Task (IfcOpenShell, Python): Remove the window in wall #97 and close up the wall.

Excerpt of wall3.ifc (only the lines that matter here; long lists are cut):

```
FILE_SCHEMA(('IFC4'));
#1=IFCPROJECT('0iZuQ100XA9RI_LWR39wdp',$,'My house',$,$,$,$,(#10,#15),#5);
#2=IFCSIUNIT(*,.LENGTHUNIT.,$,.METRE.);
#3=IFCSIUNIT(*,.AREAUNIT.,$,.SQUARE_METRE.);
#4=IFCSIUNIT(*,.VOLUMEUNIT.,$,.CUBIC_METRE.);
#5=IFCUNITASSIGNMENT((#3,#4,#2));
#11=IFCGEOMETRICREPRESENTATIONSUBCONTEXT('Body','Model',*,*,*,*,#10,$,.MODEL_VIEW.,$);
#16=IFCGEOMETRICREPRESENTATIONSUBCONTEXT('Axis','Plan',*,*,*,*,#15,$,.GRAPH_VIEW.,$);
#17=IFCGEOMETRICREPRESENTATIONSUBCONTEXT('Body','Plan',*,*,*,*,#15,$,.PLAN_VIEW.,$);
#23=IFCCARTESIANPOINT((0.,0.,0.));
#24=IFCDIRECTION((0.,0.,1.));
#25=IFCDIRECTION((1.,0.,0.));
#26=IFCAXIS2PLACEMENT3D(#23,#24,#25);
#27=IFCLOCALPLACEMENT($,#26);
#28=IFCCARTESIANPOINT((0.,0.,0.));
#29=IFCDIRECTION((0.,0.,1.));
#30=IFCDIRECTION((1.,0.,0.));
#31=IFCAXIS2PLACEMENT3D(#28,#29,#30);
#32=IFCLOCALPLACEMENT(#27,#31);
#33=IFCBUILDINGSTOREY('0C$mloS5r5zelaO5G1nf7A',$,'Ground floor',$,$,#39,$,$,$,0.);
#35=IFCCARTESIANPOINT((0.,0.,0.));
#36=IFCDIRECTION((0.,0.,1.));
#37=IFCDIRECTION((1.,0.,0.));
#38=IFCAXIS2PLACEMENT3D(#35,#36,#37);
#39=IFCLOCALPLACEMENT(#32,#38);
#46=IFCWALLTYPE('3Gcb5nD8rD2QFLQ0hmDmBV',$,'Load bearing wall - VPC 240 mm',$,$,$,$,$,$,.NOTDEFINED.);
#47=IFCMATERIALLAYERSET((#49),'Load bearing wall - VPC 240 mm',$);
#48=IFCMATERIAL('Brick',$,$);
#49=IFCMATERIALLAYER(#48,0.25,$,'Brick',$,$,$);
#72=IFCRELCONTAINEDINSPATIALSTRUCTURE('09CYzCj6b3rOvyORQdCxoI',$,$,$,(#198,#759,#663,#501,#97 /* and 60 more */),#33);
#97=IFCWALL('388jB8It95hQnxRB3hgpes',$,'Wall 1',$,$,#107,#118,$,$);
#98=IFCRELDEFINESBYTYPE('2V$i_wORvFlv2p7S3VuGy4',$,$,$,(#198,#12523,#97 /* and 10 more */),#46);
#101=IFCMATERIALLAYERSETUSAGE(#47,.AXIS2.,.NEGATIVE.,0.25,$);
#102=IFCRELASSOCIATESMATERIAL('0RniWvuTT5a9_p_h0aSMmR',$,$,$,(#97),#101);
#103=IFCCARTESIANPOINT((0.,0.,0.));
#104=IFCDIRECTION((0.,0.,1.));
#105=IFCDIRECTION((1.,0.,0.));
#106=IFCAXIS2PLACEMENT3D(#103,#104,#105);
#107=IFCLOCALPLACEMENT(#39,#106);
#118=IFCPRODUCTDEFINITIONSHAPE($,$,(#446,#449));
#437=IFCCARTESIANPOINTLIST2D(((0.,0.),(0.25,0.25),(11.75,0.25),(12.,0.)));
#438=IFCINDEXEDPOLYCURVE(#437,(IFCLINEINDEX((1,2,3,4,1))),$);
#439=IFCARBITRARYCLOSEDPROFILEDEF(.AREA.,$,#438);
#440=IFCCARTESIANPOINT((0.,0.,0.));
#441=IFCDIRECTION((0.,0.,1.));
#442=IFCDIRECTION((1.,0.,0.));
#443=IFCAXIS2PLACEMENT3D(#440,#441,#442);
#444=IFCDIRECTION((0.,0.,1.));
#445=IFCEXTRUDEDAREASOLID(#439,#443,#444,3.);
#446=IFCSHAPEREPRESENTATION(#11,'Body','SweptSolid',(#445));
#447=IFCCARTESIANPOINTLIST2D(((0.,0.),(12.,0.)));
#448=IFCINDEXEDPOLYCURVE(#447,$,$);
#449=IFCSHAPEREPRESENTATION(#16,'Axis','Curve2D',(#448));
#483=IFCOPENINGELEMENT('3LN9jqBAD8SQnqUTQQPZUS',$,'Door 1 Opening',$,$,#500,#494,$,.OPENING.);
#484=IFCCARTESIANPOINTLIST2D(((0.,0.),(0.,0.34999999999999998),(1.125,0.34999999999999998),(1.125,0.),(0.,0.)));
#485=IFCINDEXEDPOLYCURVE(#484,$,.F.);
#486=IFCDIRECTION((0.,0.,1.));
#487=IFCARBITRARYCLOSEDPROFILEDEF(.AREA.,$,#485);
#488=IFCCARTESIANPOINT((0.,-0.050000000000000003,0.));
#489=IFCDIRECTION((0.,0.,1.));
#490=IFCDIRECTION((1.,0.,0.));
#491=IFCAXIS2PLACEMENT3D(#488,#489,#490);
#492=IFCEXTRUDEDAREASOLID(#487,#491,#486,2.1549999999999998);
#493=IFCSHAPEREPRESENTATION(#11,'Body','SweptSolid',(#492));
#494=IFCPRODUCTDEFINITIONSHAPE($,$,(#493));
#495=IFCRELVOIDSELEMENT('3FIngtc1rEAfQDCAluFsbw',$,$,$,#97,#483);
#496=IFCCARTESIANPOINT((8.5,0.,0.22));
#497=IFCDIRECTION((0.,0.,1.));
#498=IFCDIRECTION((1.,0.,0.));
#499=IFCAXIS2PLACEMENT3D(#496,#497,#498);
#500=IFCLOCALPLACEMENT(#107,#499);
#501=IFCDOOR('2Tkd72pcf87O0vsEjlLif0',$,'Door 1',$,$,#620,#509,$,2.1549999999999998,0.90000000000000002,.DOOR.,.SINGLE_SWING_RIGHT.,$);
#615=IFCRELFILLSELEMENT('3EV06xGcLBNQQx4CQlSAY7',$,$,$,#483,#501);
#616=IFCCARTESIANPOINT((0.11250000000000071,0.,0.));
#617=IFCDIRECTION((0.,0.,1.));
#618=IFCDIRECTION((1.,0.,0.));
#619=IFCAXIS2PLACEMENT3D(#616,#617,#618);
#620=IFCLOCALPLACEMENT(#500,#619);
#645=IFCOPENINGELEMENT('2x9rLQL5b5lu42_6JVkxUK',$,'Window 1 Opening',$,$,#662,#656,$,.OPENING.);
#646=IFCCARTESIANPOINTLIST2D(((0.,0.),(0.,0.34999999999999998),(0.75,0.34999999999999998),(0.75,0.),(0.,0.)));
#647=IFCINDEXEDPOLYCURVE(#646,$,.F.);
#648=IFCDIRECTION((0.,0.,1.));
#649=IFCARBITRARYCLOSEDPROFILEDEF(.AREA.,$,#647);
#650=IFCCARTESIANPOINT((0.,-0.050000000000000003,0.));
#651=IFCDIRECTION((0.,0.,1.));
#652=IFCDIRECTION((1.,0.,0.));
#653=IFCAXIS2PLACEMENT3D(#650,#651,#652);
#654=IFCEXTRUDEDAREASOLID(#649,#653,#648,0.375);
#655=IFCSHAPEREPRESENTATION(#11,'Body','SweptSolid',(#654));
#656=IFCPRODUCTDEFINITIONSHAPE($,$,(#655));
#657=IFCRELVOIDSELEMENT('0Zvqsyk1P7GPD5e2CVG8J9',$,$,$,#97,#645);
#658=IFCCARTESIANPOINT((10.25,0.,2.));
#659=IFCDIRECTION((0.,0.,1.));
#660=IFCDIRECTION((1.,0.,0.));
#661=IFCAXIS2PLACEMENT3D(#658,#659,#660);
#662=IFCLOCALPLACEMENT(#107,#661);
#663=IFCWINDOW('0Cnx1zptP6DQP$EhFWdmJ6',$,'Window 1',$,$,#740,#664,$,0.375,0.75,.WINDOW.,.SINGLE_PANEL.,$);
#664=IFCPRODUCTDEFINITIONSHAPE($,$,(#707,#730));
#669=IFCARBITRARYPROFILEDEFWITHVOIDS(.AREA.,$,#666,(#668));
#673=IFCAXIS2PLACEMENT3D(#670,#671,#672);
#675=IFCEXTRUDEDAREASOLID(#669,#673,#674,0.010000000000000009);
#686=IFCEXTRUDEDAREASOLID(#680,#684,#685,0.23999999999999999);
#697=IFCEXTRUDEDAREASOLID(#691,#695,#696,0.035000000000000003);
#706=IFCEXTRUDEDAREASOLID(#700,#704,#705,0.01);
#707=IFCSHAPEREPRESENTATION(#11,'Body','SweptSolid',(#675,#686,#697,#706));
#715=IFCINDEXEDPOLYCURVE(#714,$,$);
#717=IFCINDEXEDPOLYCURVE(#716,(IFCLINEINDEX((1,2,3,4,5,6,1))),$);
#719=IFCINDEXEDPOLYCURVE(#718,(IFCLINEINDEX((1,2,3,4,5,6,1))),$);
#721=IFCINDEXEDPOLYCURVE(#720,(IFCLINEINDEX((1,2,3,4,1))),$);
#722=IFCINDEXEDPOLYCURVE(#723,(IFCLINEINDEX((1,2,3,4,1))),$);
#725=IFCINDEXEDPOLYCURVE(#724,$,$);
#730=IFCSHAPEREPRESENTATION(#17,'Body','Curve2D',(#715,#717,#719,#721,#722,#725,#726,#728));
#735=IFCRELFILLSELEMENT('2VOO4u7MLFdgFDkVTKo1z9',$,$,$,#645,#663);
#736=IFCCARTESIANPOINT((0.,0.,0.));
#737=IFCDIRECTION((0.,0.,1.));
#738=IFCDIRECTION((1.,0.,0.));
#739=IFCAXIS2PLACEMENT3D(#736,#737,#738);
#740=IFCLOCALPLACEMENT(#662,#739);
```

```python
import ifcopenshell
import ifcopenshell.api.feature
import ifcopenshell.api.root
import ifcopenshell.geom
import ifcopenshell.util.shape

model = ifcopenshell.open("wall3.ifc")
settings = ifcopenshell.geom.settings()


def volume(element):
    """Net volume in cubic metres, openings subtracted."""
    shape = ifcopenshell.geom.create_shape(settings, element)
    return ifcopenshell.util.shape.get_volume(shape.geometry)


window = model.by_guid("0Cnx1zptP6DQP$EhFWdmJ6")
opening = window.FillsVoids[0].RelatingOpeningElement
wall = opening.VoidsElements[0].RelatingBuildingElement
before = volume(wall)

ifcopenshell.api.root.remove_product(model, product=window)
ifcopenshell.api.feature.remove_feature(model, feature=opening)

after = volume(wall)

print(f"wall volume {before:.3f} -> {after:.3f} m3")

model.write("wall3-out.ifc")
```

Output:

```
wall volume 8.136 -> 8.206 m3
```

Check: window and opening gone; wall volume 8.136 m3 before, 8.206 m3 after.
